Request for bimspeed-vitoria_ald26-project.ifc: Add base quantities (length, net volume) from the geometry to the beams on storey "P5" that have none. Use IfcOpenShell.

First a look at what the model holds.

```python
import ifcopenshell
import ifcopenshell.util.element
import ifcopenshell.util.unit

model = ifcopenshell.open("bimspeed-vitoria_ald26-project.ifc")
print(model.schema)
for unit_type in ("LENGTHUNIT", "AREAUNIT", "VOLUMEUNIT"):
    print(unit_type, ifcopenshell.util.unit.calculate_unit_scale(model, unit_type))
storey = next(s for s in model.by_type("IfcBuildingStorey") if s.Name == "P5")
beams = [e for e in ifcopenshell.util.element.get_decomposition(storey) if e.is_a("IfcBeam")]
for e in sorted(beams, key=lambda e: e.id()):
    print(e.id(), e.is_a(), e.Name, list(ifcopenshell.util.element.get_psets(e, qtos_only=True)), sep=" | ")
```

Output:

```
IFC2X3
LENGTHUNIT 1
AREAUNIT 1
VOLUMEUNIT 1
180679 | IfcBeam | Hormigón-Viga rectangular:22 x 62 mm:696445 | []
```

```python
import ifcopenshell
import ifcopenshell.api.pset
import ifcopenshell.geom
import ifcopenshell.util.element
import ifcopenshell.util.shape
import ifcopenshell.util.unit

model = ifcopenshell.open("bimspeed-vitoria_ald26-project.ifc")
unit_scale = ifcopenshell.util.unit.calculate_unit_scale(model)
volume_scale = ifcopenshell.util.unit.calculate_unit_scale(model, "VOLUMEUNIT")
settings = ifcopenshell.geom.settings()

storey = next(s for s in model.by_type("IfcBuildingStorey") if s.Name == "P5")
beams = [e for e in ifcopenshell.util.element.get_decomposition(storey) if e.is_a("IfcBeam")]

for e in sorted(beams, key=lambda e: e.id()):
    if ifcopenshell.util.element.get_psets(e, qtos_only=True, should_inherit=False):
        continue
    # Geometry comes back in metres, in the element's own axes.
    shape = ifcopenshell.geom.create_shape(settings, e)
    values = {
        "Length": ifcopenshell.util.shape.get_max_xyz(shape.geometry) / unit_scale,
        "NetVolume": ifcopenshell.util.shape.get_volume(shape.geometry) / volume_scale,
    }
    qto = ifcopenshell.api.pset.add_qto(model, product=e, name="BaseQuantities")
    ifcopenshell.api.pset.edit_qto(model, qto=qto, properties=values)
    print(e.id(), {k: round(v, 3) for k, v in values.items()})

model.write("bimspeed-vitoria_ald26-project_v2.ifc")
```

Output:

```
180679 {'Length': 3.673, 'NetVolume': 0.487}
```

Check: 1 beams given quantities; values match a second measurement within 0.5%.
